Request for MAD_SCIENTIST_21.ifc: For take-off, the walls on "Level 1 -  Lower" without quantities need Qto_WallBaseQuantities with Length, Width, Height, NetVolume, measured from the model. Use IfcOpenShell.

First a look at what the model holds.

```python
import ifcopenshell
import ifcopenshell.util.element
import ifcopenshell.util.unit

model = ifcopenshell.open("MAD_SCIENTIST_21.ifc")
print(model.schema)
for unit_type in ("LENGTHUNIT", "AREAUNIT", "VOLUMEUNIT"):
    print(unit_type, ifcopenshell.util.unit.calculate_unit_scale(model, unit_type))
storey = next(s for s in model.by_type("IfcBuildingStorey") if s.Name == "Level 1 -  Lower")
walls = [e for e in ifcopenshell.util.element.get_decomposition(storey) if e.is_a("IfcWall")]
for e in sorted(walls, key=lambda e: e.id()):
    print(e.id(), e.is_a(), e.Name, list(ifcopenshell.util.element.get_psets(e, qtos_only=True)), sep=" | ")
```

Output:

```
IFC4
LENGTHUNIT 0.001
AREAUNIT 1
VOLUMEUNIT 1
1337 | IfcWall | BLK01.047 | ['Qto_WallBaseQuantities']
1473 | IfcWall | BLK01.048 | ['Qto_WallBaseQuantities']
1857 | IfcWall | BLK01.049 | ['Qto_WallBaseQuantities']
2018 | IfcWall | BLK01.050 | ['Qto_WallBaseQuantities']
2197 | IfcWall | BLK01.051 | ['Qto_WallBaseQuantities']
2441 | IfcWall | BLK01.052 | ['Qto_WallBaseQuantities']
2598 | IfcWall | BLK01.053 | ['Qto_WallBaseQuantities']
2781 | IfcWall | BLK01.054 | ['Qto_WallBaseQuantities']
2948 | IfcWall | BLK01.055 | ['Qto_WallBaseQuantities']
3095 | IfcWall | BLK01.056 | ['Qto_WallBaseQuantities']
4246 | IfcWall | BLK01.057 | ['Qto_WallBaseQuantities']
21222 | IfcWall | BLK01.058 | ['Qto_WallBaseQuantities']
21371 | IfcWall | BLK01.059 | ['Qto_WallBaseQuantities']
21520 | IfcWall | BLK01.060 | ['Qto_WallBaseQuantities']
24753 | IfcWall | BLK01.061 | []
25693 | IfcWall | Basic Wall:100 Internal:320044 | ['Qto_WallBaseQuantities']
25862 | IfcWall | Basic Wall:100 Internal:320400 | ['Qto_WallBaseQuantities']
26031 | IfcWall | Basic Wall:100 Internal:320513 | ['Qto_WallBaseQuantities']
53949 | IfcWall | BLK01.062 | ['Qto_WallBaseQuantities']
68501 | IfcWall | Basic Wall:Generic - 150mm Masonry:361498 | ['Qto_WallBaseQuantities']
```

```python
import ifcopenshell
import ifcopenshell.api.pset
import ifcopenshell.geom
import ifcopenshell.util.element
import ifcopenshell.util.shape
import ifcopenshell.util.unit

model = ifcopenshell.open("MAD_SCIENTIST_21.ifc")
unit_scale = ifcopenshell.util.unit.calculate_unit_scale(model)
volume_scale = ifcopenshell.util.unit.calculate_unit_scale(model, "VOLUMEUNIT")
settings = ifcopenshell.geom.settings()

storey = next(s for s in model.by_type("IfcBuildingStorey") if s.Name == "Level 1 -  Lower")
walls = [e for e in ifcopenshell.util.element.get_decomposition(storey) if e.is_a("IfcWall")]

for e in sorted(walls, key=lambda e: e.id()):
    if ifcopenshell.util.element.get_psets(e, qtos_only=True, should_inherit=False):
        continue
    # Geometry comes back in metres, in the element's own axes.
    shape = ifcopenshell.geom.create_shape(settings, e)
    values = {
        "Length": ifcopenshell.util.shape.get_x(shape.geometry) / unit_scale,
        "Width": ifcopenshell.util.shape.get_y(shape.geometry) / unit_scale,
        "Height": ifcopenshell.util.shape.get_z(shape.geometry) / unit_scale,
        "NetVolume": ifcopenshell.util.shape.get_volume(shape.geometry) / volume_scale,
    }
    qto = ifcopenshell.api.pset.add_qto(model, product=e, name="Qto_WallBaseQuantities")
    ifcopenshell.api.pset.edit_qto(model, qto=qto, properties=values)
    print(e.id(), {k: round(v, 3) for k, v in values.items()})

model.write("MAD_SCIENTIST_21_v2.ifc")
```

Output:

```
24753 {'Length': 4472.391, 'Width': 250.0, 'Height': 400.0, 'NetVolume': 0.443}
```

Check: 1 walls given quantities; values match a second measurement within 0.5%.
